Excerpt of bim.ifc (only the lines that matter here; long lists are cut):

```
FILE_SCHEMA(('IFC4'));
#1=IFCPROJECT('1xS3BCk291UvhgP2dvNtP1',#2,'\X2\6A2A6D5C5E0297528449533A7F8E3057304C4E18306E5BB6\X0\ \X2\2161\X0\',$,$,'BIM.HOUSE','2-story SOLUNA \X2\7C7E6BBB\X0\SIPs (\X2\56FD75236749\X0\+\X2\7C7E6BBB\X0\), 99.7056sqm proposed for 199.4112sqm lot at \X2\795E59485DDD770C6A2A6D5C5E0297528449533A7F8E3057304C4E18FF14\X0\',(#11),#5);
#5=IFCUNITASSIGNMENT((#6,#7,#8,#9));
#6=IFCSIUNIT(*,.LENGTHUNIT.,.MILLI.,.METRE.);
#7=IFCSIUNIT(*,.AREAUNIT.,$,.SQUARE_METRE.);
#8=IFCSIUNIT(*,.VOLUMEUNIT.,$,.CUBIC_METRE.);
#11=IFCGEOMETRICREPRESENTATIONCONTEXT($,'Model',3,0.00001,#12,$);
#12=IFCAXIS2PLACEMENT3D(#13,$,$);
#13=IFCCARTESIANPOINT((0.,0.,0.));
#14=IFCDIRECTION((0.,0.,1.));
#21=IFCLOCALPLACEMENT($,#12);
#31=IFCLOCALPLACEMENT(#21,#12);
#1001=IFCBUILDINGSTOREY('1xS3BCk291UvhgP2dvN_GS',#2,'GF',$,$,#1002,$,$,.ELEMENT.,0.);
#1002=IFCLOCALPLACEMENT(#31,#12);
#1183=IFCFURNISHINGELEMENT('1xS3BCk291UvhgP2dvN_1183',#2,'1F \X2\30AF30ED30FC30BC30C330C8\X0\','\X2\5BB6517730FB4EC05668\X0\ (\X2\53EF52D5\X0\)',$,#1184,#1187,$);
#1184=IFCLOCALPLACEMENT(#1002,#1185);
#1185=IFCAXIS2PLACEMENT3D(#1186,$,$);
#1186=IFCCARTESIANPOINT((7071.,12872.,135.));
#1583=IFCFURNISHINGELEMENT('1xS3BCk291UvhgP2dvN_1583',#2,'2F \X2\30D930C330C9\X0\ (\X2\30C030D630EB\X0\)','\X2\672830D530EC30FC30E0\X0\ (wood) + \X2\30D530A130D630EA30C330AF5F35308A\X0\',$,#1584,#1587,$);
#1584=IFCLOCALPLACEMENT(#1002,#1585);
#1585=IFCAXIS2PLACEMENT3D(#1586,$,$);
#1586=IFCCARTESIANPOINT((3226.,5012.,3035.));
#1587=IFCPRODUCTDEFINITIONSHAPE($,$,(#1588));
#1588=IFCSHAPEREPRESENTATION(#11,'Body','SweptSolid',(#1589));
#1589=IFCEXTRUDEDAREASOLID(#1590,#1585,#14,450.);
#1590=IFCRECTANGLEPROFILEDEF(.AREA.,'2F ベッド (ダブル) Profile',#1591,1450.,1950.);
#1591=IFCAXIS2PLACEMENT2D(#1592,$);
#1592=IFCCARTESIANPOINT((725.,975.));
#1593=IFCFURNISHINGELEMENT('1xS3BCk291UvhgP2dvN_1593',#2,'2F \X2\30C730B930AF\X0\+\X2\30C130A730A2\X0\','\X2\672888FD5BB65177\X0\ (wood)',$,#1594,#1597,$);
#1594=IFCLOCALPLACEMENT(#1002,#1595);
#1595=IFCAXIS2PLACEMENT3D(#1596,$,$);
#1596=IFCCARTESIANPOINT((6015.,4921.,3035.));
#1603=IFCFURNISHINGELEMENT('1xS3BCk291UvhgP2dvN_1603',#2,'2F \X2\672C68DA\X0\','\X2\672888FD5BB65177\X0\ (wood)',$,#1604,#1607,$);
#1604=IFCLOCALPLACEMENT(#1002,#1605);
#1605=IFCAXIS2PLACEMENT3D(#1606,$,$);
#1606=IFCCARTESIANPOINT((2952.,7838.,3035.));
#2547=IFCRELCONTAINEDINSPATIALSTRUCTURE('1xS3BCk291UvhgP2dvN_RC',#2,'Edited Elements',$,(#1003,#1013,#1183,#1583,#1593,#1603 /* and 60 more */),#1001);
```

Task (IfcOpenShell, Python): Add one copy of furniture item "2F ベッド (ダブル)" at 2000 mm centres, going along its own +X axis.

```python
import ifcopenshell
import ifcopenshell.api.geometry
import ifcopenshell.api.root
import ifcopenshell.util.element
import ifcopenshell.util.placement
import ifcopenshell.util.unit

model = ifcopenshell.open("bim.ifc")
unit_scale = ifcopenshell.util.unit.calculate_unit_scale(model)


def reuse_history(source, copy):
    """copy_class also copies each property set's owner history, people and application; keep the originals."""
    for rel in copy.IsDefinedBy:
        if rel.is_a("IfcRelDefinesByProperties") and (history := rel.RelatingPropertyDefinition.OwnerHistory):
            rel.RelatingPropertyDefinition.OwnerHistory = source.OwnerHistory
            ifcopenshell.util.element.remove_deep2(model, history)


source = model.by_id(1583)
base = ifcopenshell.util.placement.get_local_placement(source.ObjectPlacement)
step = base[:3, 0] * 2 / unit_scale

for i in range(1, 2):
    copy = ifcopenshell.api.root.copy_class(model, product=source)
    copy.Representation = ifcopenshell.util.element.copy_deep(
        model, source.Representation, exclude=["IfcGeometricRepresentationContext", "IfcRepresentationMap"]
    )
    reuse_history(source, copy)
    matrix = base.copy()
    matrix[:3, 3] += i * step
    print("added at", matrix[:3, 3].round(3) + 0.0)
    ifcopenshell.api.geometry.edit_object_placement(model, product=copy, matrix=matrix, is_si=False)

model.write("bim_v2.ifc")
```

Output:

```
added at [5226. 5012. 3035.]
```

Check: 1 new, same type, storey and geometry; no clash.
